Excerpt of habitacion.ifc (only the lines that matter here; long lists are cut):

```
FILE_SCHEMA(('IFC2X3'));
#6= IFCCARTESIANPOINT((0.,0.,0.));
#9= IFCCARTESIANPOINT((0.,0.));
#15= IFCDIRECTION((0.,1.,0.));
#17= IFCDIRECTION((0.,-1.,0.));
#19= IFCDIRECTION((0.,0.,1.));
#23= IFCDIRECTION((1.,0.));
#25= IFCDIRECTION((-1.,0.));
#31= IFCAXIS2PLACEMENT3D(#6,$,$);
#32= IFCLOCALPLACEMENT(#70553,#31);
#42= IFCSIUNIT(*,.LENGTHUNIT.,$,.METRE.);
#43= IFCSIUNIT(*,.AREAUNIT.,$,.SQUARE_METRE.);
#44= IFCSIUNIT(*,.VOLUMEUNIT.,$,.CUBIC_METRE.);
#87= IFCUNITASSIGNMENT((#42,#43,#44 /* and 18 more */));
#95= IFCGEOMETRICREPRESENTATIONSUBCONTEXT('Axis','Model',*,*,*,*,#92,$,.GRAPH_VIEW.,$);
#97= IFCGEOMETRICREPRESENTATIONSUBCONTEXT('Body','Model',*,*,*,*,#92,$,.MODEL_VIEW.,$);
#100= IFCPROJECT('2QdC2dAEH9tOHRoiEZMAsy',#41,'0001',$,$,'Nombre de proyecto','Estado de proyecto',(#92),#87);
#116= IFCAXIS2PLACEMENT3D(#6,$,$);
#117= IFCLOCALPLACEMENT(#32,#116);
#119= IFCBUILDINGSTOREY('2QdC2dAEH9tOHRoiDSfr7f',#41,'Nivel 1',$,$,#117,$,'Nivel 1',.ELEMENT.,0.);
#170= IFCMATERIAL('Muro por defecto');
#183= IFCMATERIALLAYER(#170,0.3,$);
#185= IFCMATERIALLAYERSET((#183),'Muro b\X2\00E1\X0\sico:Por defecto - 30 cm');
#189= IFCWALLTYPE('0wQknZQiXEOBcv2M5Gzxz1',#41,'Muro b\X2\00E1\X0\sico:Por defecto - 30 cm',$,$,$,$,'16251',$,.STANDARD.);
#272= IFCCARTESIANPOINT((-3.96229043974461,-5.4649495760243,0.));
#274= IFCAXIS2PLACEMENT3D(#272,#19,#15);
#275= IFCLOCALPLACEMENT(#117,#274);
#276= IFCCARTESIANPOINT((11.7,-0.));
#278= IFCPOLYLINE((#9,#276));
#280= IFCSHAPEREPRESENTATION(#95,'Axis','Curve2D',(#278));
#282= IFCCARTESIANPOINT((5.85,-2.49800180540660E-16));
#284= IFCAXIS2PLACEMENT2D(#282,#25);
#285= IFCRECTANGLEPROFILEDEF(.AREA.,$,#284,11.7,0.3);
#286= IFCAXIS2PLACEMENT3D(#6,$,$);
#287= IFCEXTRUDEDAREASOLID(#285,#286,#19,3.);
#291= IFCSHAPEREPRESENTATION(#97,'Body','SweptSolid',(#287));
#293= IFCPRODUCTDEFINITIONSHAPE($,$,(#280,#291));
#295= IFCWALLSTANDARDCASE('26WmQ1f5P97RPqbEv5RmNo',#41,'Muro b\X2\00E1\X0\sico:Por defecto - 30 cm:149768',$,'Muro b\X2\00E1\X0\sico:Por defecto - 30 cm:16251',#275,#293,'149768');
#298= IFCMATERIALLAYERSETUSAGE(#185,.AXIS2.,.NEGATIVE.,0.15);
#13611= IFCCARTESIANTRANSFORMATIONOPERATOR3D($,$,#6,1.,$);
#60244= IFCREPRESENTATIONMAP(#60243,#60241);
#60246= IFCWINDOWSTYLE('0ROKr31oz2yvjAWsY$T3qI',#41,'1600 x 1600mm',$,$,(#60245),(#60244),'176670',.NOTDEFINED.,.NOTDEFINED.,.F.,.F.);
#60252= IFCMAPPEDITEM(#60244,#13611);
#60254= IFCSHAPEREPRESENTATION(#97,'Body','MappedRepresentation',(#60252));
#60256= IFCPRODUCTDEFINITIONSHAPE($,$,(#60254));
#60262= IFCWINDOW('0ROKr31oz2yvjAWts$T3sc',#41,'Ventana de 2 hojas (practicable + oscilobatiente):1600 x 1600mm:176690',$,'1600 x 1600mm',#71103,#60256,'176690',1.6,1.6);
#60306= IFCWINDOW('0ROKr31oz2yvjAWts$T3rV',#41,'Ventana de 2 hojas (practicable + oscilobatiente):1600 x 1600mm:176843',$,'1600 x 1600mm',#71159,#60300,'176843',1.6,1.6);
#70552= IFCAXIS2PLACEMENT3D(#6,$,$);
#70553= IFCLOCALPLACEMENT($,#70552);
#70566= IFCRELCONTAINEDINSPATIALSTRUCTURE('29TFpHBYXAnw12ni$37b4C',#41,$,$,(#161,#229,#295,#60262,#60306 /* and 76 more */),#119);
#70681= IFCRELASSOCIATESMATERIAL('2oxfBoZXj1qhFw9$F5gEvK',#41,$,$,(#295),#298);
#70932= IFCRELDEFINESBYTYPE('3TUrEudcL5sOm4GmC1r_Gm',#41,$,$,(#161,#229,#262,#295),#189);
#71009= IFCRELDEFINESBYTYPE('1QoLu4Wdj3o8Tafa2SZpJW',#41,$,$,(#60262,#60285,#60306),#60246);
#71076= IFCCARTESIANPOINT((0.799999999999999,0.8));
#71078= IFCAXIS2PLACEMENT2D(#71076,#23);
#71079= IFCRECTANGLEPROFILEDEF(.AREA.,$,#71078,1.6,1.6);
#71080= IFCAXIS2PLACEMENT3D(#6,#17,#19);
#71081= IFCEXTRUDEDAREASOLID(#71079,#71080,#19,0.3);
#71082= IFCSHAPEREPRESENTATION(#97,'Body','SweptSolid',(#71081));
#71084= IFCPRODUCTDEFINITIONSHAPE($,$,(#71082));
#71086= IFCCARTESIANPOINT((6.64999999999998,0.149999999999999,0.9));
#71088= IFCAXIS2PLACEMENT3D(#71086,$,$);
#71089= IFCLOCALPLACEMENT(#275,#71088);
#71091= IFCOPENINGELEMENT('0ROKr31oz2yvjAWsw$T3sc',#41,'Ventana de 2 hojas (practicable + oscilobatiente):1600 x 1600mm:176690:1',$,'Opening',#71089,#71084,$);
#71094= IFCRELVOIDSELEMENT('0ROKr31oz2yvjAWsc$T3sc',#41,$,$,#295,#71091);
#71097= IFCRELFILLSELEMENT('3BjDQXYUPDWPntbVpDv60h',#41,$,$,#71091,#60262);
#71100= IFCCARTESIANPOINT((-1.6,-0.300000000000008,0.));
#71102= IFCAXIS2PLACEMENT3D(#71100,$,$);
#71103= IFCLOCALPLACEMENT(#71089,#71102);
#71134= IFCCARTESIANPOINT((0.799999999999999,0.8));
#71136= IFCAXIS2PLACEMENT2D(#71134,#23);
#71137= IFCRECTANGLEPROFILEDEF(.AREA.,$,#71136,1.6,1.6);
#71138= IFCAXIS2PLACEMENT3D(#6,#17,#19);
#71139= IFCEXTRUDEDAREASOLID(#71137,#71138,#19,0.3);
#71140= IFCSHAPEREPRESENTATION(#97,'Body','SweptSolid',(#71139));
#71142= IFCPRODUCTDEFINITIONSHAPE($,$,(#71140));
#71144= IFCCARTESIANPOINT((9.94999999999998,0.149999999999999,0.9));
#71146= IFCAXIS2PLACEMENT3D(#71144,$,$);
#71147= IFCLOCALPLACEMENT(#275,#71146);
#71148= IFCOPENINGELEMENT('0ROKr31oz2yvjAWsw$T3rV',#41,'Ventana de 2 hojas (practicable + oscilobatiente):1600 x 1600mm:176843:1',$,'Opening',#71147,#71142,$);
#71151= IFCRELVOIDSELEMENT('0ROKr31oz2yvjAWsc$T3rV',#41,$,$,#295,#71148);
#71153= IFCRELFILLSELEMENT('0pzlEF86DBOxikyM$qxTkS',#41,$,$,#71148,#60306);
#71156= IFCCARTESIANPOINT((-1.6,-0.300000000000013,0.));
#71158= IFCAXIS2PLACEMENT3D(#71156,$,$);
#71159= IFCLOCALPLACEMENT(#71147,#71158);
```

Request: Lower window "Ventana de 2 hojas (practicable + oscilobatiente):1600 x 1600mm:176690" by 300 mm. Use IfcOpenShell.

```python
import numpy as np
import ifcopenshell
import ifcopenshell.api.geometry
import ifcopenshell.util.placement
import ifcopenshell.util.unit

model = ifcopenshell.open("habitacion.ifc")
unit_scale = ifcopenshell.util.unit.calculate_unit_scale(model)

window = model.by_guid("0ROKr31oz2yvjAWts$T3sc")
opening = window.FillsVoids[0].RelatingOpeningElement
dz = -0.3

shift = np.array([0.0, 0.0, dz])
# The window is placed relative to its opening, so it follows when the opening moves.
matrix = ifcopenshell.util.placement.get_local_placement(opening.ObjectPlacement)
matrix[:3, 3] += shift
ifcopenshell.api.geometry.edit_object_placement(
    model, product=opening, matrix=matrix, is_si=False, should_transform_children=True
)

print(f"moved by {dz * unit_scale:+.3f} m")

model.write("habitacion_updated.ifc")
```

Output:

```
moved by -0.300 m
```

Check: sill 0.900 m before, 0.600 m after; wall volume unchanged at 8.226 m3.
